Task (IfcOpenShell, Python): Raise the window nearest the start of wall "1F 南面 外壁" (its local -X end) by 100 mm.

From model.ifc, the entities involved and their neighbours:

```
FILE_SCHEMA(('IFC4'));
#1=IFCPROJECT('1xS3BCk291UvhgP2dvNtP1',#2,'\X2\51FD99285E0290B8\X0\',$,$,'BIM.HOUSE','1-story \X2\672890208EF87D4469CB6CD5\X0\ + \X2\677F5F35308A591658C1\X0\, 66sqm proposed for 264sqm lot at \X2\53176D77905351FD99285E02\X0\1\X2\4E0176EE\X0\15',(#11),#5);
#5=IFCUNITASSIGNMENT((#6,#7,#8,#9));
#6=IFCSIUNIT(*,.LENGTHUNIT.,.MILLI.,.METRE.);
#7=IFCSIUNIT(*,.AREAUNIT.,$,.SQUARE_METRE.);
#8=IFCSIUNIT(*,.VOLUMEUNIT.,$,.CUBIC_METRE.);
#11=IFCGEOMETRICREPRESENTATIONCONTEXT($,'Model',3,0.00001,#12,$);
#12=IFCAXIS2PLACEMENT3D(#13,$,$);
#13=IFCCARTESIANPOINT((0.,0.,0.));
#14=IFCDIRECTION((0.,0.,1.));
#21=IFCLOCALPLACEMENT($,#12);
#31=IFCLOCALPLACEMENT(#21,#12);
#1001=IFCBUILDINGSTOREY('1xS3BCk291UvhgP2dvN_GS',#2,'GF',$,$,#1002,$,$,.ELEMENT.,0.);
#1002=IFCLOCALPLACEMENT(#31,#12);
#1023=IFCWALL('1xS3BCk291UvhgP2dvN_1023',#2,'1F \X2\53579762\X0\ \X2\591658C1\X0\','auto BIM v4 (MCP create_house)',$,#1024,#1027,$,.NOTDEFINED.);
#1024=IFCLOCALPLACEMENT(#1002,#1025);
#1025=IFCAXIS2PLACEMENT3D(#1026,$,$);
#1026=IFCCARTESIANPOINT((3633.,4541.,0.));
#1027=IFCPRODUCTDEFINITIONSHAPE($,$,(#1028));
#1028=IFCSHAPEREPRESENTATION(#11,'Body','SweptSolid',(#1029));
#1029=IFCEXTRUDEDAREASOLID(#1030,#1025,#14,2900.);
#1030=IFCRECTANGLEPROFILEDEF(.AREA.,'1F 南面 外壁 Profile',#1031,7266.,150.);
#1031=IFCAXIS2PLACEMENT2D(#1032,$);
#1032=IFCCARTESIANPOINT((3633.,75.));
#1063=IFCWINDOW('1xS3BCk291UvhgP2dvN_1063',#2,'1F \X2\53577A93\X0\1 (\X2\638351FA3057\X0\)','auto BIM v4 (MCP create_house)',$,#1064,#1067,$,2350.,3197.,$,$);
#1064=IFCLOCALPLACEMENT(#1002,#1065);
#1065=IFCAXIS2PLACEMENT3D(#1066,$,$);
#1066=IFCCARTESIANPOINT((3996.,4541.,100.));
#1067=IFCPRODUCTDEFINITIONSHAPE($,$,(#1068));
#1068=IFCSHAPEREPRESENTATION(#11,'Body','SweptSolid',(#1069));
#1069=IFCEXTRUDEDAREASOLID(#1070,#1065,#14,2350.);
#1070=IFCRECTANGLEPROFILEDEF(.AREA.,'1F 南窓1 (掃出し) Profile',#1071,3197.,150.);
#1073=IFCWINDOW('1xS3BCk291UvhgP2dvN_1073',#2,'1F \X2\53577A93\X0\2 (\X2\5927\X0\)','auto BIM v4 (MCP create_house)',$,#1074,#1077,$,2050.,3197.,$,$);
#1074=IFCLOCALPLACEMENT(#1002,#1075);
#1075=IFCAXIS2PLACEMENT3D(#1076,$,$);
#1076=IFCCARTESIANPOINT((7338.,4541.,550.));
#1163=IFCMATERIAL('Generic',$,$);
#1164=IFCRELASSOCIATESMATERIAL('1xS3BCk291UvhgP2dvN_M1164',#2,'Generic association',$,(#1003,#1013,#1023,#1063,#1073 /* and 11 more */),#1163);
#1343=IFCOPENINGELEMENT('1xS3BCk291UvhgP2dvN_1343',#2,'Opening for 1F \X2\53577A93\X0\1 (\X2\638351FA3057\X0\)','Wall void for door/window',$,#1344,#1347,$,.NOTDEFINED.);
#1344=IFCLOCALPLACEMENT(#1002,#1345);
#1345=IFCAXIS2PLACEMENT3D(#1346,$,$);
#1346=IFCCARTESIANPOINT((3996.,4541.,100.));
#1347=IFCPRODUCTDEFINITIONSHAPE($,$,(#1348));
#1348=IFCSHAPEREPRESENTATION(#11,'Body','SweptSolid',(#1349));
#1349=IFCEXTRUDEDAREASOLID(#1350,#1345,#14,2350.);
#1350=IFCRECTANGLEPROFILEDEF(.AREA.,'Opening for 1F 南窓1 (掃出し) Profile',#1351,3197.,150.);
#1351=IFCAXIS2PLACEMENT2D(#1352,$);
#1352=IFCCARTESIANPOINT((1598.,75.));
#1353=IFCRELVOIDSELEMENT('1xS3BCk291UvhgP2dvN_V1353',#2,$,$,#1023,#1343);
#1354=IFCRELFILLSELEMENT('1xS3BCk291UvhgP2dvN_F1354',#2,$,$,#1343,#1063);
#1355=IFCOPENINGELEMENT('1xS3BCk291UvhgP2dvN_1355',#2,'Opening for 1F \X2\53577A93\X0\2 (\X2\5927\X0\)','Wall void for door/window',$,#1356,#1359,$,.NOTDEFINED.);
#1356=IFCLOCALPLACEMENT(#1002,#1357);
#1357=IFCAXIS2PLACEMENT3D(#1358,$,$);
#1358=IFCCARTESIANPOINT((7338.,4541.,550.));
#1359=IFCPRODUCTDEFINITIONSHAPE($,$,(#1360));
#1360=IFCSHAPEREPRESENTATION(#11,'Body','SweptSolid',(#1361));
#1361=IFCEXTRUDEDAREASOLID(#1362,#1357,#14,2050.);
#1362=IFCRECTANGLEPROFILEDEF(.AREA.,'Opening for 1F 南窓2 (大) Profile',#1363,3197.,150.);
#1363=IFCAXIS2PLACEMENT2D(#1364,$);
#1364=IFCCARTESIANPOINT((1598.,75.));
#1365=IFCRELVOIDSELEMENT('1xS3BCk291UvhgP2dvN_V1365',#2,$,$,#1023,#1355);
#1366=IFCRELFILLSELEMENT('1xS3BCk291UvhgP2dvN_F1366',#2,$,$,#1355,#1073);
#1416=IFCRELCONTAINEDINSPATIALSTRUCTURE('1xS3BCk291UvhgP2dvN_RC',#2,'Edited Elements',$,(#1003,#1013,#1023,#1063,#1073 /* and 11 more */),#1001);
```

```python
import numpy as np
import ifcopenshell
import ifcopenshell.api.geometry
import ifcopenshell.util.placement
import ifcopenshell.util.unit

model = ifcopenshell.open("model.ifc")
unit_scale = ifcopenshell.util.unit.calculate_unit_scale(model)

window = model.by_id(1063)
opening = window.FillsVoids[0].RelatingOpeningElement
dz = 0.1 / unit_scale

shift = np.array([0.0, 0.0, dz])
# The window is not placed relative to its opening, so move both.
for product in (opening, window):
    matrix = ifcopenshell.util.placement.get_local_placement(product.ObjectPlacement)
    matrix[:3, 3] += shift
    ifcopenshell.api.geometry.edit_object_placement(model, product=product, matrix=matrix, is_si=False)

print(f"moved by {dz * unit_scale:+.3f} m")

model.write("model_v2.ifc")
```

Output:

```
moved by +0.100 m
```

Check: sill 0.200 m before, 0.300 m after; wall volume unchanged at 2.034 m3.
